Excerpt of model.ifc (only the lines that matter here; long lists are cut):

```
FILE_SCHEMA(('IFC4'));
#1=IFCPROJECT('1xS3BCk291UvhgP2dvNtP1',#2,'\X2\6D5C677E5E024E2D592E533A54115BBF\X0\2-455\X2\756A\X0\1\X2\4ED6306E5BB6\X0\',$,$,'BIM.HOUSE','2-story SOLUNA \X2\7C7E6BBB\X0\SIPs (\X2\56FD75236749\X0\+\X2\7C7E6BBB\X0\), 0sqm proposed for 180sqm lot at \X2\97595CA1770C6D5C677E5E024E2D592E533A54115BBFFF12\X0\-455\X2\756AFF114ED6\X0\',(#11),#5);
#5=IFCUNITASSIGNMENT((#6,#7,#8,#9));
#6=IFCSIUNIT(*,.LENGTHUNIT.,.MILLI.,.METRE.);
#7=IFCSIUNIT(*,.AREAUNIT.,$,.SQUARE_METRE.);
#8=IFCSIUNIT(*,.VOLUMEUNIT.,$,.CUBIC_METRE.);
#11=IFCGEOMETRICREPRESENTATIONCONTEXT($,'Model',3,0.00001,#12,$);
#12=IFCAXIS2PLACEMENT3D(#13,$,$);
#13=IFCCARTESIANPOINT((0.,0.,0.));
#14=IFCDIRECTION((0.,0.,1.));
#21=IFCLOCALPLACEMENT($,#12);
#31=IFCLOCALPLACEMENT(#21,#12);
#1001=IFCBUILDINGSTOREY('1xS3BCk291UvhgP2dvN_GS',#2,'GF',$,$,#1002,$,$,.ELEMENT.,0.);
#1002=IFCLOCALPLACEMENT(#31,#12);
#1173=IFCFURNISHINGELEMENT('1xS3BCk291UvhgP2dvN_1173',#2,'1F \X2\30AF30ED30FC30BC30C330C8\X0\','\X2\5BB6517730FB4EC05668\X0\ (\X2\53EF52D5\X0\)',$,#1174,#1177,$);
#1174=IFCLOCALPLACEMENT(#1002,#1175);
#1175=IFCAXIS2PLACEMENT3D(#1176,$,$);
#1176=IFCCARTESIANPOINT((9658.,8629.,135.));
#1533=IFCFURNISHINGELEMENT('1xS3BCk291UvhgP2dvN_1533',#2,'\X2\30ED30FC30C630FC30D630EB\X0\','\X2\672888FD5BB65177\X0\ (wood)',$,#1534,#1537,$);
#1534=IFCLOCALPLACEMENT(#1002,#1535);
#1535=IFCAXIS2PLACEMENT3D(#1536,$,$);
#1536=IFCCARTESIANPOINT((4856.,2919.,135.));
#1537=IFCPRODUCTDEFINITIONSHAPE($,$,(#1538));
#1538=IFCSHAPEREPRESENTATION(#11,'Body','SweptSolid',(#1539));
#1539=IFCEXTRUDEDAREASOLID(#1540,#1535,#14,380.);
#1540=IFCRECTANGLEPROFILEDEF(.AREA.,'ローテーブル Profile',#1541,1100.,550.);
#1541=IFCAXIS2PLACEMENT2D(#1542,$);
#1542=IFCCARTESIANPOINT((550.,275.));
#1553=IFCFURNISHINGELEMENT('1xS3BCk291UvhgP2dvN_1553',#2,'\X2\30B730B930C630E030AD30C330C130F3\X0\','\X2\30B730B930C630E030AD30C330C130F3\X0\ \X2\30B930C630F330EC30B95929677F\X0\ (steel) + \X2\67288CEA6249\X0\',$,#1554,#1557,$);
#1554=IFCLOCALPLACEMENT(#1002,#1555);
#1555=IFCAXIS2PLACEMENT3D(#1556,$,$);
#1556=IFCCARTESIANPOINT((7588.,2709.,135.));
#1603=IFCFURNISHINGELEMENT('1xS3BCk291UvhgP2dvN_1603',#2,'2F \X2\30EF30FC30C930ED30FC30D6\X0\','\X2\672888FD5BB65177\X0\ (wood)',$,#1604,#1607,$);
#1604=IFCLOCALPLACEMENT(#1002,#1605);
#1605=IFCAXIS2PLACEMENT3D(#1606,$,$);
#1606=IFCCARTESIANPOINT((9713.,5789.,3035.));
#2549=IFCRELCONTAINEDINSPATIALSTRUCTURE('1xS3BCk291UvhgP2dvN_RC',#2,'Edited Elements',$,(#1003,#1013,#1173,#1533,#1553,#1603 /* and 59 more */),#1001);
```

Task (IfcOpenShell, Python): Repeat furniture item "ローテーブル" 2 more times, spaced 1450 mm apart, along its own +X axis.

```python
import ifcopenshell
import ifcopenshell.api.geometry
import ifcopenshell.api.root
import ifcopenshell.util.element
import ifcopenshell.util.placement
import ifcopenshell.util.unit

model = ifcopenshell.open("model.ifc")
unit_scale = ifcopenshell.util.unit.calculate_unit_scale(model)


def reuse_history(source, copy):
    """copy_class also copies each property set's owner history, people and application; keep the originals."""
    for rel in copy.IsDefinedBy:
        if rel.is_a("IfcRelDefinesByProperties") and (history := rel.RelatingPropertyDefinition.OwnerHistory):
            rel.RelatingPropertyDefinition.OwnerHistory = source.OwnerHistory
            ifcopenshell.util.element.remove_deep2(model, history)


source = model.by_guid("1xS3BCk291UvhgP2dvN_1533")
base = ifcopenshell.util.placement.get_local_placement(source.ObjectPlacement)
step = base[:3, 0] * 1.45 / unit_scale

for i in range(1, 3):
    copy = ifcopenshell.api.root.copy_class(model, product=source)
    copy.Representation = ifcopenshell.util.element.copy_deep(
        model, source.Representation, exclude=["IfcGeometricRepresentationContext", "IfcRepresentationMap"]
    )
    reuse_history(source, copy)
    matrix = base.copy()
    matrix[:3, 3] += i * step
    print("added at", matrix[:3, 3].round(3) + 0.0)
    ifcopenshell.api.geometry.edit_object_placement(model, product=copy, matrix=matrix, is_si=False)

model.write("model_updated.ifc")
```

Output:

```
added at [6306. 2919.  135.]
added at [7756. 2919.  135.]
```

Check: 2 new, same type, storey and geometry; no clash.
